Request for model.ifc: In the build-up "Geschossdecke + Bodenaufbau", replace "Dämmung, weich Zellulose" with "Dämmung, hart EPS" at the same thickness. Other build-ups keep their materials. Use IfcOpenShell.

First a look at what the model holds.

```python
import ifcopenshell
import ifcopenshell.util.element

model = ifcopenshell.open("model.ifc")
print(model.schema)
for layer_set in model.by_type("IfcMaterialLayerSet"):
    if layer_set.LayerSetName == "Geschossdecke + Bodenaufbau":
        for layer in layer_set.MaterialLayers:
            print(layer.id(), layer.Material and layer.Material.Name, layer.LayerThickness, sep=" | ")
        print(len(ifcopenshell.util.element.get_elements_by_material(model, layer_set)), "elements and types use it")
print(sorted(m.Name for m in model.by_type("IfcMaterial") if m.Name)[:60])
```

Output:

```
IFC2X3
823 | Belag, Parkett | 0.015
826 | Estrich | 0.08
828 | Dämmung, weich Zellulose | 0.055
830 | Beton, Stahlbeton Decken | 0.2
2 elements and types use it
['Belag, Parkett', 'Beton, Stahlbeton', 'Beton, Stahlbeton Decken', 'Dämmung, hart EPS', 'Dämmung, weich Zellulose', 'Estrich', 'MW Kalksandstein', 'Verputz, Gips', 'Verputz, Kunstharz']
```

```python
import ifcopenshell
import ifcopenshell.api.material

model = ifcopenshell.open("model.ifc")

layer_set = next(s for s in model.by_type("IfcMaterialLayerSet") if s.LayerSetName == "Geschossdecke + Bodenaufbau")
layer = next(l for l in layer_set.MaterialLayers if l.Material and l.Material.Name == "Dämmung, weich Zellulose")
material = next(m for m in model.by_type("IfcMaterial") if m.Name == "Dämmung, hart EPS")

# Point this one layer at the other material; renaming the old one would change it everywhere.
ifcopenshell.api.material.edit_layer(model, layer=layer, attributes={}, material=material)

print([l.Material.Name if l.Material else None for l in layer_set.MaterialLayers])

model.write("model_edited.ifc")
```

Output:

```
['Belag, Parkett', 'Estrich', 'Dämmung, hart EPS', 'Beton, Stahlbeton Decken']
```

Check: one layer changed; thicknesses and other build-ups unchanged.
